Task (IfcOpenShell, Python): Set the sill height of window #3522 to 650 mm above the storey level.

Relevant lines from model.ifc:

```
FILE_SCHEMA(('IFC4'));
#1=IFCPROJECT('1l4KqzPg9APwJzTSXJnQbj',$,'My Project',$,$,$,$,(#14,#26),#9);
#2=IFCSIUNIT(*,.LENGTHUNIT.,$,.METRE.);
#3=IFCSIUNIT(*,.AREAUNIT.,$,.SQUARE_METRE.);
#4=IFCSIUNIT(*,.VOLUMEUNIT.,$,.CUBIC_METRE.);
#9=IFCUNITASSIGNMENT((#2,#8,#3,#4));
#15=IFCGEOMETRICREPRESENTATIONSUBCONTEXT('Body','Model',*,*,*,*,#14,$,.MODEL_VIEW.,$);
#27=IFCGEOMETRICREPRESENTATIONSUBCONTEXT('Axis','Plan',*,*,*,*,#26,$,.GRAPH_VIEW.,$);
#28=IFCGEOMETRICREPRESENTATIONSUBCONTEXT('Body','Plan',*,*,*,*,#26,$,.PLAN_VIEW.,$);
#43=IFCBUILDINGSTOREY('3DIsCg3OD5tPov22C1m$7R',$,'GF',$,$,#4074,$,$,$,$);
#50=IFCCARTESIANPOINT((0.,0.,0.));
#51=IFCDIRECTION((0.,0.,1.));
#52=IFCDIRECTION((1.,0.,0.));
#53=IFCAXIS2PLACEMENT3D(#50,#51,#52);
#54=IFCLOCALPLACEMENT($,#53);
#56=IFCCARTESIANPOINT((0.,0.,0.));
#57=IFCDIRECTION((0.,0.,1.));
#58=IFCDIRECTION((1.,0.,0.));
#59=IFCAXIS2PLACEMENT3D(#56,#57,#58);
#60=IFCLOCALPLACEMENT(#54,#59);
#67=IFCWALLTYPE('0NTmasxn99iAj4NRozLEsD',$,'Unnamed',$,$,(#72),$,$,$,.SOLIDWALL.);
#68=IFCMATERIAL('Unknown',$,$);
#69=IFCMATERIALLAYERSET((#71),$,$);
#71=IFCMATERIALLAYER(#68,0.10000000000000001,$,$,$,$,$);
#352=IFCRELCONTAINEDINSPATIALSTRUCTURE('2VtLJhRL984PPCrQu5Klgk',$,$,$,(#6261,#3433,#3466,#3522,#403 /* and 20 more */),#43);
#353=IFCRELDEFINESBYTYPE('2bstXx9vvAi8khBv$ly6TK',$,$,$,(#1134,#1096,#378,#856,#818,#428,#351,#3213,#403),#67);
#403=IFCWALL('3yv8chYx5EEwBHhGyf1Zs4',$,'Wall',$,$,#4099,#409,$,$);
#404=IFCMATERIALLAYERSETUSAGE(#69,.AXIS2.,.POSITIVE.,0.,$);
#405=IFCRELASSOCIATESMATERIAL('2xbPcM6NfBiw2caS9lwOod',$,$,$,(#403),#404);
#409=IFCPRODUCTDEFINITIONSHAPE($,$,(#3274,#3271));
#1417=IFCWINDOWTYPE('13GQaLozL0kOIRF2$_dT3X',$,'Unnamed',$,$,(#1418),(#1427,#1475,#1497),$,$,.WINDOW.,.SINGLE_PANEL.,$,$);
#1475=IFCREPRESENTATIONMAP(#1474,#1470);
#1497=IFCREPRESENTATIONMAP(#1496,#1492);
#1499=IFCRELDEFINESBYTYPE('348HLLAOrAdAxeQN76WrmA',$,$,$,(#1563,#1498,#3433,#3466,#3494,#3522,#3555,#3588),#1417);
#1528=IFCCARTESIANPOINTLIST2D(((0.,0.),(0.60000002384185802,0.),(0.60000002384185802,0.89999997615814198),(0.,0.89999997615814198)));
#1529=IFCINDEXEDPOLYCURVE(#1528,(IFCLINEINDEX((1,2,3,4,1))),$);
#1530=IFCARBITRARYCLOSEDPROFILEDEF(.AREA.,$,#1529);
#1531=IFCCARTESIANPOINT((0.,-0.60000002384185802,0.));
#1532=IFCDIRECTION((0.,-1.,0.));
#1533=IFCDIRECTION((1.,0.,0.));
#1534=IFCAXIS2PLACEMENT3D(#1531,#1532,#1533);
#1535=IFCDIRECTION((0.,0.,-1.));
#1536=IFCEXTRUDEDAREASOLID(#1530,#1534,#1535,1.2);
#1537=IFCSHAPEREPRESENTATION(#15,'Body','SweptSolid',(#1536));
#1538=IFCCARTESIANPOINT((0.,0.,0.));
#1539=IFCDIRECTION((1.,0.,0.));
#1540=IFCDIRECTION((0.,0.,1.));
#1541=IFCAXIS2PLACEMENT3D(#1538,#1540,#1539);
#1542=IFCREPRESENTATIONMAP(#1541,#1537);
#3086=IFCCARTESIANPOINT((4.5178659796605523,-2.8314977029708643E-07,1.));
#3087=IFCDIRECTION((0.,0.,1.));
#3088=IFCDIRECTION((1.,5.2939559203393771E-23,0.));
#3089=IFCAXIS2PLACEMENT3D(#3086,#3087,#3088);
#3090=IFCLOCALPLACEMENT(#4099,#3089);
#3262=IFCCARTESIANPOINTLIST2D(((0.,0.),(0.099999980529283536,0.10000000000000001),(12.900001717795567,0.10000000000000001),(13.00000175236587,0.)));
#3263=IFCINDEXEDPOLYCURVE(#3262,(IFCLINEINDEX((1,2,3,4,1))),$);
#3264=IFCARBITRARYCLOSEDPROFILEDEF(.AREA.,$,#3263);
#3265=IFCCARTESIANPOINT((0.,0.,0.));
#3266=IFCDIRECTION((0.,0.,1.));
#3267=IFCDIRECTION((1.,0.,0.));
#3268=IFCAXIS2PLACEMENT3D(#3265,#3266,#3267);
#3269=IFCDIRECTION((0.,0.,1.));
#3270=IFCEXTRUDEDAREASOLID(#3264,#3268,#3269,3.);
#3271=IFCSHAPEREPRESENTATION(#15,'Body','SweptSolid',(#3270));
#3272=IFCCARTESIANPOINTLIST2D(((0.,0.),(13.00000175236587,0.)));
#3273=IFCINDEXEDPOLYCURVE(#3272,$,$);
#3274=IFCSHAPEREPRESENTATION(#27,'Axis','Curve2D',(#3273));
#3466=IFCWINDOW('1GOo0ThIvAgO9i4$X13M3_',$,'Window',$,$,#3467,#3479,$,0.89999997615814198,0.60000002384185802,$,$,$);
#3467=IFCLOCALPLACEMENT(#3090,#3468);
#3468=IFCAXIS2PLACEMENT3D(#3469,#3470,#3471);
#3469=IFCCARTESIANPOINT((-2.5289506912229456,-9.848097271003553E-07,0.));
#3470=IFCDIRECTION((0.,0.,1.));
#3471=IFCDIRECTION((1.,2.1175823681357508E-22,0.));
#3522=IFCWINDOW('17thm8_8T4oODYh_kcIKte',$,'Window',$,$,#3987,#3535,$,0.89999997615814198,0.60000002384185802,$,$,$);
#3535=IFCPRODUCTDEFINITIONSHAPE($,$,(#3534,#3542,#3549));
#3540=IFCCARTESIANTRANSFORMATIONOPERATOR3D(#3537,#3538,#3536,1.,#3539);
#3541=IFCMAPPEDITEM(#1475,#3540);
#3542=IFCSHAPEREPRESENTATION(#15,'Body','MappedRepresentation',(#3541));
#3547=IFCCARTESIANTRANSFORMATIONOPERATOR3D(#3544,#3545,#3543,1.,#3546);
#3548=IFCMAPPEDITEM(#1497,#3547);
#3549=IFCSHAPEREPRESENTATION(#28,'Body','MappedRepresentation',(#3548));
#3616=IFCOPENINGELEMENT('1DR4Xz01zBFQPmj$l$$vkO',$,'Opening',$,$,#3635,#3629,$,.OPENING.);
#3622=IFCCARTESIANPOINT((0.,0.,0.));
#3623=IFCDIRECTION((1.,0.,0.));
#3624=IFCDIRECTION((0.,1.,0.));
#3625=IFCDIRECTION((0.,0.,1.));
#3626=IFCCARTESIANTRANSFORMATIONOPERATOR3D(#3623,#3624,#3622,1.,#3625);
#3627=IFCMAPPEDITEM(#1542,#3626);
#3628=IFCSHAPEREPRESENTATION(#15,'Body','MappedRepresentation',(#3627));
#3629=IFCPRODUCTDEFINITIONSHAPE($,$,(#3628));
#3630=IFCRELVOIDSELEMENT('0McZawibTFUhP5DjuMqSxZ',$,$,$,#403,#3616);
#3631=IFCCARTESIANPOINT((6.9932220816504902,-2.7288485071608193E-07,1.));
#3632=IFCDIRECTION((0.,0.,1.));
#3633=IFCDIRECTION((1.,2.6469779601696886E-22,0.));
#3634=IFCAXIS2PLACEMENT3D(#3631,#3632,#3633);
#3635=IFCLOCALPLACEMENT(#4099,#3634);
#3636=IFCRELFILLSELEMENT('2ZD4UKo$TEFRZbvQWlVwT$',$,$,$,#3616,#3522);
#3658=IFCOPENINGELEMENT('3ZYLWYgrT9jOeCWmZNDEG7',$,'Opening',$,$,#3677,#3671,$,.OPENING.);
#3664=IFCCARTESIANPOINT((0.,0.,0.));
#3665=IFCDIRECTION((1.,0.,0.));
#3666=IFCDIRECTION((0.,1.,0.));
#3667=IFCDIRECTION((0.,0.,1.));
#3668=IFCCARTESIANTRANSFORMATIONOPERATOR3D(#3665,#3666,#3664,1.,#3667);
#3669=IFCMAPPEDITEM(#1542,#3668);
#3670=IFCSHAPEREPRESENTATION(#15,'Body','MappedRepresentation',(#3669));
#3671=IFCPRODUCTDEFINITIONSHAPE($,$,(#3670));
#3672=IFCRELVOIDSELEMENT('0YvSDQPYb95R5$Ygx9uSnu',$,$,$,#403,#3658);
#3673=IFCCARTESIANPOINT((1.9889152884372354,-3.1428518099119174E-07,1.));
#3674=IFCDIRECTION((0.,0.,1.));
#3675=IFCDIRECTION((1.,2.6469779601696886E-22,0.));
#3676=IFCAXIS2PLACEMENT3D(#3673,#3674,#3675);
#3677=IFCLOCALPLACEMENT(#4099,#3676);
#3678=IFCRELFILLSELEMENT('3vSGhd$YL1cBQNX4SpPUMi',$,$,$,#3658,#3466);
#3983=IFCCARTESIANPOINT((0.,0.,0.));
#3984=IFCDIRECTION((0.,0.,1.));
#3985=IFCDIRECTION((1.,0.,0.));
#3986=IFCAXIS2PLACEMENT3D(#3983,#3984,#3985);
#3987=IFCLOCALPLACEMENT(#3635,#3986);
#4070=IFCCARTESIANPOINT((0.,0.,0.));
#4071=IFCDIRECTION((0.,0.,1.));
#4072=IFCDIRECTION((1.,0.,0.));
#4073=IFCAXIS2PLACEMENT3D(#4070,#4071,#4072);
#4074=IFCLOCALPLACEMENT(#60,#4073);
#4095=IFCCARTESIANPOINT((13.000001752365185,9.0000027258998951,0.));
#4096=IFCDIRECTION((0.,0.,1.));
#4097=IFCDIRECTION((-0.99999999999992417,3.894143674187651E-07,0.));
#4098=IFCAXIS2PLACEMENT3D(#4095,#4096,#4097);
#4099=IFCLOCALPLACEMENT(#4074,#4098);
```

```python
import numpy as np
import ifcopenshell
import ifcopenshell.api.geometry
import ifcopenshell.geom
import ifcopenshell.util.element
import ifcopenshell.util.placement
import ifcopenshell.util.shape
import ifcopenshell.util.unit

model = ifcopenshell.open("model.ifc")
unit_scale = ifcopenshell.util.unit.calculate_unit_scale(model)

window = model.by_guid("17thm8_8T4oODYh_kcIKte")
opening = window.FillsVoids[0].RelatingOpeningElement
storey = ifcopenshell.util.element.get_container(window, ifc_class="IfcBuildingStorey")
level = ifcopenshell.util.placement.get_local_placement(storey.ObjectPlacement)[2, 3]

# The opening's origin need not be at the sill, so measure its lowest point.
shape = ifcopenshell.geom.create_shape(ifcopenshell.geom.settings(), opening)
bottom = ifcopenshell.util.shape.get_shape_bottom_elevation(shape, shape.geometry) / unit_scale
dz = level + 0.65 - bottom

shift = np.array([0.0, 0.0, dz])
# The window is placed relative to its opening, so it follows when the opening moves.
matrix = ifcopenshell.util.placement.get_local_placement(opening.ObjectPlacement)
matrix[:3, 3] += shift
ifcopenshell.api.geometry.edit_object_placement(
    model, product=opening, matrix=matrix, is_si=False, should_transform_children=True
)

print(f"moved by {dz * unit_scale:+.3f} m")

model.write("model_updated.ifc")
```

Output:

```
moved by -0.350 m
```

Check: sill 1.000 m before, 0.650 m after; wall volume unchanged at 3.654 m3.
